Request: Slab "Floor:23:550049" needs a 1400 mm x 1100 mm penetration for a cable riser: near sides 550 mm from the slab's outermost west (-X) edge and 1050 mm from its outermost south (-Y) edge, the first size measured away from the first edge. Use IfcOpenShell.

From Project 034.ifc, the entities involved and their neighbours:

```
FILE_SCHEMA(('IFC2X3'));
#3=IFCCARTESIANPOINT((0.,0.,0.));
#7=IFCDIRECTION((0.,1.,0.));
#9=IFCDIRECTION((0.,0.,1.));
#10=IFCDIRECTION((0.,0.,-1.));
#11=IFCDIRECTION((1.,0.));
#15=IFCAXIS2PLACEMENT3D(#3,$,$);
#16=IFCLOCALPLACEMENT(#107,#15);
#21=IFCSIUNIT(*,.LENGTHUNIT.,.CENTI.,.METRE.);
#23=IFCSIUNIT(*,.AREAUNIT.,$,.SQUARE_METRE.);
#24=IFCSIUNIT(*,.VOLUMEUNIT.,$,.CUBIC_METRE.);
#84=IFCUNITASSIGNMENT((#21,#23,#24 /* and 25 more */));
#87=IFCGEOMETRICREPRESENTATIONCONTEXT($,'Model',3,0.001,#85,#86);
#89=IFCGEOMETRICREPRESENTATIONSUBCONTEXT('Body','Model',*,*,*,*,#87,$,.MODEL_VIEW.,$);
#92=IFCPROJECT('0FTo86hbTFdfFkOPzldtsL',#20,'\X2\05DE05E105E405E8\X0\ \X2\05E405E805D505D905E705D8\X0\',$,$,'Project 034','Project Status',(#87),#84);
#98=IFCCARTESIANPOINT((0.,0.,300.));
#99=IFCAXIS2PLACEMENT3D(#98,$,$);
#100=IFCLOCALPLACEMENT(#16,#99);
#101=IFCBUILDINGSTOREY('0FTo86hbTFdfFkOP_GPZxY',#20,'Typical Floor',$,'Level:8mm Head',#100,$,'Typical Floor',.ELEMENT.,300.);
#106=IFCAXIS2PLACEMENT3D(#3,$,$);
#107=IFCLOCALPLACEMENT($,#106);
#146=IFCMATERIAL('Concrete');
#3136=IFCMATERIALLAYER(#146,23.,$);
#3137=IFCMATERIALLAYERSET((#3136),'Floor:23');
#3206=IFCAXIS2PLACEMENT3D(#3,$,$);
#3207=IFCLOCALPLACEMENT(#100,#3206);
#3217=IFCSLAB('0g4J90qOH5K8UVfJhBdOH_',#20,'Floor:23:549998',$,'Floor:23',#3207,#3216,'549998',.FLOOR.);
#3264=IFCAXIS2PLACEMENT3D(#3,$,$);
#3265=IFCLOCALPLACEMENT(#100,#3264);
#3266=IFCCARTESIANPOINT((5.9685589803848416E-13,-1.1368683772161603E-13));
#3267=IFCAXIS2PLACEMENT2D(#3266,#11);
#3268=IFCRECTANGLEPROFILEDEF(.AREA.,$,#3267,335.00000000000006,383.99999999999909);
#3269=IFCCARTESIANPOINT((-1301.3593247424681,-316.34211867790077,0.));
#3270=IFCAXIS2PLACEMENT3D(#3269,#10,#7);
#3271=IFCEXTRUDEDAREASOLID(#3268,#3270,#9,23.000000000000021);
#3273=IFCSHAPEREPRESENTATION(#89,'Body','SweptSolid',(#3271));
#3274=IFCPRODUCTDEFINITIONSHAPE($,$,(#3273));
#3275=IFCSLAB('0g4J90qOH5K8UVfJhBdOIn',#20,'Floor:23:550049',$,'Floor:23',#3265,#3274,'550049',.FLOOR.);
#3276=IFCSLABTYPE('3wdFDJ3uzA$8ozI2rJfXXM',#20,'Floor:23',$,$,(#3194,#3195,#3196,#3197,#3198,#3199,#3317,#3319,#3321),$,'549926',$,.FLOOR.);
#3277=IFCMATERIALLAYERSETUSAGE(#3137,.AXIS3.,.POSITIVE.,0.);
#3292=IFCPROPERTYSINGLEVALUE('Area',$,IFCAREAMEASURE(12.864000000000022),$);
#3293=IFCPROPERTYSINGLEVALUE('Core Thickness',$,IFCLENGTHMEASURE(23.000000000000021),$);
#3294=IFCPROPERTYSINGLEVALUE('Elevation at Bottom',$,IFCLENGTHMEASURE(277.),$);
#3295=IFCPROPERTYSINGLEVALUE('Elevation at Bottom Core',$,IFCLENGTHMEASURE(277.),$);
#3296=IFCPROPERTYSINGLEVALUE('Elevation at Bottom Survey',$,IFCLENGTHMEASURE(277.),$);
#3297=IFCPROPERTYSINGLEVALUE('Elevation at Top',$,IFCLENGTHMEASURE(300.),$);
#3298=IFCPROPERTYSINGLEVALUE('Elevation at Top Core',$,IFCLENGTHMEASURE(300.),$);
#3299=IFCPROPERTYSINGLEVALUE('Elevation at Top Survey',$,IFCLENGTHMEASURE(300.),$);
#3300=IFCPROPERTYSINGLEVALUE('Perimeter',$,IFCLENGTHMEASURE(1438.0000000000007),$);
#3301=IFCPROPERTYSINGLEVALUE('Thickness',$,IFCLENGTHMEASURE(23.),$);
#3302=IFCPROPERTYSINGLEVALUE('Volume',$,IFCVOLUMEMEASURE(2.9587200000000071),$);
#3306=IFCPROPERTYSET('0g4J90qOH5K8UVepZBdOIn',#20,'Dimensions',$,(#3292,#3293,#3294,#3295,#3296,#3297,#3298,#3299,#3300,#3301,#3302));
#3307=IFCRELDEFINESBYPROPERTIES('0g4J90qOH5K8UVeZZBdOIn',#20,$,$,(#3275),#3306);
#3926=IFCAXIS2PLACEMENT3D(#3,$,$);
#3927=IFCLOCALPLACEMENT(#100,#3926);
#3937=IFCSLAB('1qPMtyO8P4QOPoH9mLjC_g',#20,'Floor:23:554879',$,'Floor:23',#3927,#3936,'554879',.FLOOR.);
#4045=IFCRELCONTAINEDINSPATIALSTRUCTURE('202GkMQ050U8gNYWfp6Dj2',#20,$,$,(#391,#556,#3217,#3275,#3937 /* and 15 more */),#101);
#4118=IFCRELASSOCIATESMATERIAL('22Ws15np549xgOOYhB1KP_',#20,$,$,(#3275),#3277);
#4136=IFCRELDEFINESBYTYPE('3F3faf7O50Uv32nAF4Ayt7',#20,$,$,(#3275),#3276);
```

```python
import numpy as np
import ifcopenshell
import ifcopenshell.api.feature
import ifcopenshell.api.geometry
import ifcopenshell.api.pset
import ifcopenshell.api.root
import ifcopenshell.geom
import ifcopenshell.util.element
import ifcopenshell.util.placement
import ifcopenshell.util.representation
import ifcopenshell.util.shape
import ifcopenshell.util.unit

model = ifcopenshell.open("Project 034.ifc")
unit_scale = ifcopenshell.util.unit.calculate_unit_scale(model)
area_scale = ifcopenshell.util.unit.calculate_unit_scale(model, "AREAUNIT")
volume_scale = ifcopenshell.util.unit.calculate_unit_scale(model, "VOLUMEUNIT")
settings = ifcopenshell.geom.settings()


def volume(element):
    """Net volume in cubic metres, openings subtracted."""
    shape = ifcopenshell.geom.create_shape(settings, element)
    return ifcopenshell.util.shape.get_volume(shape.geometry)


slab = model.by_id(3275)
before = volume(slab)

# Extent in the slab's own axes, in metres. The edges named are its -X and -Y sides.
slab_shape = ifcopenshell.geom.create_shape(settings, slab)
vertices = ifcopenshell.util.shape.get_vertices(slab_shape.geometry)
x_min, y_min, bottom = vertices.min(axis=0)
top = vertices[:, 2].max()

opening = ifcopenshell.api.root.create_entity(model, ifc_class="IfcOpeningElement", name="Cable riser opening")
context = ifcopenshell.util.representation.get_context(model, "Model", "Body", "MODEL_VIEW")
width, depth = 1.4, 1.1
outline = [(0.0, 0.0), (width, 0.0), (width, depth), (0.0, depth), (0.0, 0.0)]
# Overshoot both faces by 50 mm so the cut is clean.
shape = ifcopenshell.api.geometry.add_slab_representation(
    model, context=context, depth=top - bottom + 0.1, polyline=outline
)
ifcopenshell.api.geometry.assign_representation(model, product=opening, representation=shape)

matrix = ifcopenshell.util.placement.get_local_placement(slab.ObjectPlacement)
matrix[:, 3] = matrix @ np.append(np.array([x_min + 0.55, y_min + 1.05, bottom - 0.05]) / unit_scale, 1.0)
ifcopenshell.api.geometry.edit_object_placement(model, product=opening, matrix=matrix, is_si=False)
ifcopenshell.api.feature.add_feature(model, feature=opening, element=slab)

after = volume(slab)

# Update the slab's stored quantities.
pset = model.by_id(ifcopenshell.util.element.get_pset(slab, "Dimensions", should_inherit=False)["id"])
ifcopenshell.api.pset.edit_pset(model, pset=pset, properties={
    "Area": model.create_entity("IfcAreaMeasure", after / (top - bottom) / area_scale),
    "Volume": model.create_entity("IfcVolumeMeasure", after / volume_scale),
})

print(f"slab volume {before:.3f} -> {after:.3f} m3")

model.write("Project 034-out.ifc")
```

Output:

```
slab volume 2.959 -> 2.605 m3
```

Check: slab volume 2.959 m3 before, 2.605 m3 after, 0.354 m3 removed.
